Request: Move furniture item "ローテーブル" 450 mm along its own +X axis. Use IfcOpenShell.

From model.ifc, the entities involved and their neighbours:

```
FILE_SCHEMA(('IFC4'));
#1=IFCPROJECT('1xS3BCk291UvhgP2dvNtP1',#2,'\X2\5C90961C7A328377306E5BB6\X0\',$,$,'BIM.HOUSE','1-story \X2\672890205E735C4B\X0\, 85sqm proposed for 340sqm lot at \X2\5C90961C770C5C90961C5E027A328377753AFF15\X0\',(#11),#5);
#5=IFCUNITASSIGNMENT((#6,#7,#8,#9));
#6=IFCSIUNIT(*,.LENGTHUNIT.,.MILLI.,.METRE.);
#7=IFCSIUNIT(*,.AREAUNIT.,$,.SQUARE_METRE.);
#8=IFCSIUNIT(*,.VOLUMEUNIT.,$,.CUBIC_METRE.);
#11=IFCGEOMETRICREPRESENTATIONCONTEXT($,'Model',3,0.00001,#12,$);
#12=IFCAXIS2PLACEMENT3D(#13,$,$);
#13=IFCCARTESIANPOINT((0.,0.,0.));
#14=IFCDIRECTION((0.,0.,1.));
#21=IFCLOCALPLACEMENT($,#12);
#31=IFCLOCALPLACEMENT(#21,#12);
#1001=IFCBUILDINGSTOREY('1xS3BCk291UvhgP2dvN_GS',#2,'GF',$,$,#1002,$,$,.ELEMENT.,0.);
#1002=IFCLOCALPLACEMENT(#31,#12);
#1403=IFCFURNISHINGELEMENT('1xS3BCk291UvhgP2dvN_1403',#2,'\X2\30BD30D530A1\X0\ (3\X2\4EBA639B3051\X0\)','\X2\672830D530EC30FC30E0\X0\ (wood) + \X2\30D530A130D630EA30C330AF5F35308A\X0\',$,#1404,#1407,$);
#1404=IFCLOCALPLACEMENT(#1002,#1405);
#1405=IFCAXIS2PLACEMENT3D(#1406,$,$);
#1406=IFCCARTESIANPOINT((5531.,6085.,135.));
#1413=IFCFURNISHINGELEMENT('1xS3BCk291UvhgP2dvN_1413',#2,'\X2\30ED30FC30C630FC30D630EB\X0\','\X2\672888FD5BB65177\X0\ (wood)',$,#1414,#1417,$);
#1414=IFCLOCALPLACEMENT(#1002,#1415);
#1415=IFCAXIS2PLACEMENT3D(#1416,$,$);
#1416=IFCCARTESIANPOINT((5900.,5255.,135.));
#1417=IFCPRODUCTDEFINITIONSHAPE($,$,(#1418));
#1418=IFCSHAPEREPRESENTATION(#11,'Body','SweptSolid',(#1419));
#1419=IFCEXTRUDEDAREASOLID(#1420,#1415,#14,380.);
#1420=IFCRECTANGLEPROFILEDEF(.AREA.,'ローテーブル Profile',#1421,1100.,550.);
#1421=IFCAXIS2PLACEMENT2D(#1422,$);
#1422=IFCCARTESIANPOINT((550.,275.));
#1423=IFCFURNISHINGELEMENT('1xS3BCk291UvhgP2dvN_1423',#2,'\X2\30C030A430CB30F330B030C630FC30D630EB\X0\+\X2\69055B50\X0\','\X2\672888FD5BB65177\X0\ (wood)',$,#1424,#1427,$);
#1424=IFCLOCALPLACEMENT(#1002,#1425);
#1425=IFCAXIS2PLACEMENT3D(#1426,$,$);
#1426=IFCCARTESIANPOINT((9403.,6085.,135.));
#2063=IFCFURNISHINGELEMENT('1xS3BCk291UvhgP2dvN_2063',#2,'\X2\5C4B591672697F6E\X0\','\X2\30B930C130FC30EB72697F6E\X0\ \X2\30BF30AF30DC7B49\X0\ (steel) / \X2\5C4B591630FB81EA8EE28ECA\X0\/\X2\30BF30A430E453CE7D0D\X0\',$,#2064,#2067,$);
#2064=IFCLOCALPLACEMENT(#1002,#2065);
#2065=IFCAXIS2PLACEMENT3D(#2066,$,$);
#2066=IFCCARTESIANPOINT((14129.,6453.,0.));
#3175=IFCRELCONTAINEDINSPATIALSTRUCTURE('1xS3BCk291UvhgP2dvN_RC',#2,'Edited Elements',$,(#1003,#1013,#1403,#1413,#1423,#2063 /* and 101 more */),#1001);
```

```python
import ifcopenshell
import ifcopenshell.api.geometry
import ifcopenshell.util.placement
import ifcopenshell.util.unit

model = ifcopenshell.open("model.ifc")
unit_scale = ifcopenshell.util.unit.calculate_unit_scale(model)

item = model.by_guid("1xS3BCk291UvhgP2dvN_1413")
matrix = ifcopenshell.util.placement.get_local_placement(item.ObjectPlacement)
matrix[:3, 3] += matrix[:3, 0] * 0.45 / unit_scale
ifcopenshell.api.geometry.edit_object_placement(model, product=item, matrix=matrix, is_si=False)

print(ifcopenshell.util.placement.get_local_placement(item.ObjectPlacement).round(3) + 0.0)

model.write("model_updated.ifc")
```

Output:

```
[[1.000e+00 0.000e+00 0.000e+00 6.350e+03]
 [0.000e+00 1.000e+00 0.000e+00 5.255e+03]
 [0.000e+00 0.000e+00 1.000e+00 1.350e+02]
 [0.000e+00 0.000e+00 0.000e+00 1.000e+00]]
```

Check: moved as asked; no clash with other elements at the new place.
